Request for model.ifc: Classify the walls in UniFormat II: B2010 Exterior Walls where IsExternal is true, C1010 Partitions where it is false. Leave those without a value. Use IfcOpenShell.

First a look at what the model holds.

```python
import ifcopenshell
import ifcopenshell.util.element

model = ifcopenshell.open("model.ifc")
print(model.schema)
print("classifications:", [c.Name for c in model.by_type("IfcClassification")])
values = [ifcopenshell.util.element.get_pset(e, "Pset_WallCommon", "IsExternal") for e in model.by_type("IfcWall")]
for value in (True, False, None):
    print("IsExternal", value, values.count(value))
```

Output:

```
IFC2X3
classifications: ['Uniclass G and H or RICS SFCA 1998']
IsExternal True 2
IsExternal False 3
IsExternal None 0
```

```python
import ifcopenshell
import ifcopenshell.api.classification
import ifcopenshell.util.element

model = ifcopenshell.open("model.ifc")

# IFC2X3 requires Source and Edition and has no link from the project to the system.
system = model.create_entity("IfcClassification", Source="ASTM", Edition="E1557", Name="UniFormat II")

walls = model.by_type("IfcWall")
external = {e: ifcopenshell.util.element.get_pset(e, "Pset_WallCommon", "IsExternal") for e in walls}
for flag, code, name in ((True, "B2010", "Exterior Walls"), (False, "C1010", "Partitions")):
    products = [e for e in walls if external[e] is flag]
    ifcopenshell.api.classification.add_reference(
        model, products=products, classification=system, identification=code, name=name
    )
    print(code, len(products))

model.write("model_rev.ifc")
```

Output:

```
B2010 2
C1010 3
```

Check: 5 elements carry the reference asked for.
